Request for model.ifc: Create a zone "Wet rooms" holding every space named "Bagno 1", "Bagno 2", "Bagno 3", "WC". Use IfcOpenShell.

First a look at what the model holds.

```python
import ifcopenshell

model = ifcopenshell.open("model.ifc")
print(model.schema)
seen = {}
for space in model.by_type("IfcSpace"):
    seen[space.LongName] = seen.get(space.LongName, 0) + 1
for name, count in sorted(seen.items(), key=str):
    print(count, "x", name)
print("zones:", [z.Name for z in model.by_type("IfcZone")][:20])
```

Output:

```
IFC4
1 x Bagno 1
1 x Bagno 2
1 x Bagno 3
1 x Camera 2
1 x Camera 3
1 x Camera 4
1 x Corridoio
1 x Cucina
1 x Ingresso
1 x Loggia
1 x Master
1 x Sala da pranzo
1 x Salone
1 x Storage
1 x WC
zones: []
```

```python
import ifcopenshell
import ifcopenshell.api.group
import ifcopenshell.api.root

model = ifcopenshell.open("model.ifc")

names = {"Bagno 1", "Bagno 2", "Bagno 3", "WC"}
spaces = [s for s in model.by_type("IfcSpace") if s.LongName in names]

zone = ifcopenshell.api.root.create_entity(model, ifc_class="IfcZone", name="Wet rooms")
ifcopenshell.api.group.assign_group(model, products=spaces, group=zone)
print(len(spaces), "spaces in", zone.Name)

model.write("model_edited.ifc")
```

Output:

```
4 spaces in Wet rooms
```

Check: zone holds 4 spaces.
